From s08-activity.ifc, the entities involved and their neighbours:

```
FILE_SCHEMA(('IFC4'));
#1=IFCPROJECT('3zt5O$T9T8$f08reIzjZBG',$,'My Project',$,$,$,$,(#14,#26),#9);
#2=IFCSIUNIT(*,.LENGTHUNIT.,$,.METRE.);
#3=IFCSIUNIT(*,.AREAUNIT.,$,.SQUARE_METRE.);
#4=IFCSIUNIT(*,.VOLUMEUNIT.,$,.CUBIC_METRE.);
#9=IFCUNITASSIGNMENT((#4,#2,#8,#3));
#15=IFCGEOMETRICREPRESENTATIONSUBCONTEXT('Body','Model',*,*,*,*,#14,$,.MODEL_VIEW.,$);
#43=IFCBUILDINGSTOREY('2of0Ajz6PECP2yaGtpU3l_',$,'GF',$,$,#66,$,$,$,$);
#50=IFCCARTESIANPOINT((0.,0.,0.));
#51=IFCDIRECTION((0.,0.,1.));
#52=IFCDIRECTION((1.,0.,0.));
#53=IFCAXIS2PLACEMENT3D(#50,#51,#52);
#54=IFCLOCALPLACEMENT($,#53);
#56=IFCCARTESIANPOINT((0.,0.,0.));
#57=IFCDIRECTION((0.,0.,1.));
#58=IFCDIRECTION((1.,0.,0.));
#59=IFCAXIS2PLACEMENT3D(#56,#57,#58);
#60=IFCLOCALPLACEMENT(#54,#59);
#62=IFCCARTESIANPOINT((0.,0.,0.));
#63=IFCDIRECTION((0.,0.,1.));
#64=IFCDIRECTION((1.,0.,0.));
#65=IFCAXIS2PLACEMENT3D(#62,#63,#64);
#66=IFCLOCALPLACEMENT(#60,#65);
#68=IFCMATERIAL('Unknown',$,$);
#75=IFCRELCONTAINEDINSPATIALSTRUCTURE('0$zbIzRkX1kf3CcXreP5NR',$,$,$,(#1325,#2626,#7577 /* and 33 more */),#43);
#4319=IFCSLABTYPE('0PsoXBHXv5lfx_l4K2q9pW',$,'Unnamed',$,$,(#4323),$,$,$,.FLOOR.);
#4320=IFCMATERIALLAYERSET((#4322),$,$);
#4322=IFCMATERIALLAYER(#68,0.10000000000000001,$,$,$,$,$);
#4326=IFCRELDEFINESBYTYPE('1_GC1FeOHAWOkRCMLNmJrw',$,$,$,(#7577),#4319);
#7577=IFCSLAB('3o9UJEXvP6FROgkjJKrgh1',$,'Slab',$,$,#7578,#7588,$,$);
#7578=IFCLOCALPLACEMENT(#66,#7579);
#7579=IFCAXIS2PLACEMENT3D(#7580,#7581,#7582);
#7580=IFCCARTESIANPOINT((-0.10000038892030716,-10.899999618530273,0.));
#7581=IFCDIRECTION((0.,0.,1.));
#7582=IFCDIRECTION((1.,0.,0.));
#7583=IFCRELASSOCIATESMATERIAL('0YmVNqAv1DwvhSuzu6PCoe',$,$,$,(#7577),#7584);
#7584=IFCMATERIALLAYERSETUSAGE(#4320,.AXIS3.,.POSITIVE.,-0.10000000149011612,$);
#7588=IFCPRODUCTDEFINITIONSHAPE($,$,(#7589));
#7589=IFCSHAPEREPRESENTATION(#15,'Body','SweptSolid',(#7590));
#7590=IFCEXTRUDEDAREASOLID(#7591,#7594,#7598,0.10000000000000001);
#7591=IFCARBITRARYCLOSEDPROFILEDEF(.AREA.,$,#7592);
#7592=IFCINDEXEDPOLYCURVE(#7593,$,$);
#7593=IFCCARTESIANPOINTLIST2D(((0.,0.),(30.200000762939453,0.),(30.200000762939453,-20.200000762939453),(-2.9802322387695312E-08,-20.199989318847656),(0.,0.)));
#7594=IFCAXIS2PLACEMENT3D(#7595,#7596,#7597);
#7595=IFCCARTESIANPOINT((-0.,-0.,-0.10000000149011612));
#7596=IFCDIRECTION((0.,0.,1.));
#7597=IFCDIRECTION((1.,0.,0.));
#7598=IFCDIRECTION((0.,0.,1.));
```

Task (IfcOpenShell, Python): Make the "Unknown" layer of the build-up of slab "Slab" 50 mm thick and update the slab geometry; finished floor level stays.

```python
import ifcopenshell
import ifcopenshell.util.element
import ifcopenshell.util.representation
import ifcopenshell.util.unit

model = ifcopenshell.open("s08-activity.ifc")
unit_scale = ifcopenshell.util.unit.calculate_unit_scale(model)

layer_set = model.by_id(4320)
layer = next(l for l in layer_set.MaterialLayers if l.Material and l.Material.Name == "Unknown")
change = 0.05 / unit_scale - layer.LayerThickness
layer.LayerThickness += change

# Geometry does not follow the layer set by itself.
slabs = [e for e in ifcopenshell.util.element.get_elements_by_material(model, layer_set) if e.is_a("IfcSlab")]
for slab in sorted(slabs, key=lambda e: e.id()):
    body = ifcopenshell.util.representation.get_representation(slab, "Model", "Body")
    solid = body.Items[0]
    old_depth = solid.Depth
    solid.Depth += change
    # Extruded upwards: lower the start of the extrusion so the top stays.
    x, y, z = solid.Position.Location.Coordinates
    solid.Position.Location = model.createIfcCartesianPoint((x, y, z - change))
    print(slab.id(), f"{old_depth:g} -> {solid.Depth:g}")

# The layers are counted up from the underside, which has moved.
for usage in {ifcopenshell.util.element.get_material(slab) for slab in slabs}:
    usage.OffsetFromReferenceLine -= change

model.write("s08-activity_rev.ifc")
```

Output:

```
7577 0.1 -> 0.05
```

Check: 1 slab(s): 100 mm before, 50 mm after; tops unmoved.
